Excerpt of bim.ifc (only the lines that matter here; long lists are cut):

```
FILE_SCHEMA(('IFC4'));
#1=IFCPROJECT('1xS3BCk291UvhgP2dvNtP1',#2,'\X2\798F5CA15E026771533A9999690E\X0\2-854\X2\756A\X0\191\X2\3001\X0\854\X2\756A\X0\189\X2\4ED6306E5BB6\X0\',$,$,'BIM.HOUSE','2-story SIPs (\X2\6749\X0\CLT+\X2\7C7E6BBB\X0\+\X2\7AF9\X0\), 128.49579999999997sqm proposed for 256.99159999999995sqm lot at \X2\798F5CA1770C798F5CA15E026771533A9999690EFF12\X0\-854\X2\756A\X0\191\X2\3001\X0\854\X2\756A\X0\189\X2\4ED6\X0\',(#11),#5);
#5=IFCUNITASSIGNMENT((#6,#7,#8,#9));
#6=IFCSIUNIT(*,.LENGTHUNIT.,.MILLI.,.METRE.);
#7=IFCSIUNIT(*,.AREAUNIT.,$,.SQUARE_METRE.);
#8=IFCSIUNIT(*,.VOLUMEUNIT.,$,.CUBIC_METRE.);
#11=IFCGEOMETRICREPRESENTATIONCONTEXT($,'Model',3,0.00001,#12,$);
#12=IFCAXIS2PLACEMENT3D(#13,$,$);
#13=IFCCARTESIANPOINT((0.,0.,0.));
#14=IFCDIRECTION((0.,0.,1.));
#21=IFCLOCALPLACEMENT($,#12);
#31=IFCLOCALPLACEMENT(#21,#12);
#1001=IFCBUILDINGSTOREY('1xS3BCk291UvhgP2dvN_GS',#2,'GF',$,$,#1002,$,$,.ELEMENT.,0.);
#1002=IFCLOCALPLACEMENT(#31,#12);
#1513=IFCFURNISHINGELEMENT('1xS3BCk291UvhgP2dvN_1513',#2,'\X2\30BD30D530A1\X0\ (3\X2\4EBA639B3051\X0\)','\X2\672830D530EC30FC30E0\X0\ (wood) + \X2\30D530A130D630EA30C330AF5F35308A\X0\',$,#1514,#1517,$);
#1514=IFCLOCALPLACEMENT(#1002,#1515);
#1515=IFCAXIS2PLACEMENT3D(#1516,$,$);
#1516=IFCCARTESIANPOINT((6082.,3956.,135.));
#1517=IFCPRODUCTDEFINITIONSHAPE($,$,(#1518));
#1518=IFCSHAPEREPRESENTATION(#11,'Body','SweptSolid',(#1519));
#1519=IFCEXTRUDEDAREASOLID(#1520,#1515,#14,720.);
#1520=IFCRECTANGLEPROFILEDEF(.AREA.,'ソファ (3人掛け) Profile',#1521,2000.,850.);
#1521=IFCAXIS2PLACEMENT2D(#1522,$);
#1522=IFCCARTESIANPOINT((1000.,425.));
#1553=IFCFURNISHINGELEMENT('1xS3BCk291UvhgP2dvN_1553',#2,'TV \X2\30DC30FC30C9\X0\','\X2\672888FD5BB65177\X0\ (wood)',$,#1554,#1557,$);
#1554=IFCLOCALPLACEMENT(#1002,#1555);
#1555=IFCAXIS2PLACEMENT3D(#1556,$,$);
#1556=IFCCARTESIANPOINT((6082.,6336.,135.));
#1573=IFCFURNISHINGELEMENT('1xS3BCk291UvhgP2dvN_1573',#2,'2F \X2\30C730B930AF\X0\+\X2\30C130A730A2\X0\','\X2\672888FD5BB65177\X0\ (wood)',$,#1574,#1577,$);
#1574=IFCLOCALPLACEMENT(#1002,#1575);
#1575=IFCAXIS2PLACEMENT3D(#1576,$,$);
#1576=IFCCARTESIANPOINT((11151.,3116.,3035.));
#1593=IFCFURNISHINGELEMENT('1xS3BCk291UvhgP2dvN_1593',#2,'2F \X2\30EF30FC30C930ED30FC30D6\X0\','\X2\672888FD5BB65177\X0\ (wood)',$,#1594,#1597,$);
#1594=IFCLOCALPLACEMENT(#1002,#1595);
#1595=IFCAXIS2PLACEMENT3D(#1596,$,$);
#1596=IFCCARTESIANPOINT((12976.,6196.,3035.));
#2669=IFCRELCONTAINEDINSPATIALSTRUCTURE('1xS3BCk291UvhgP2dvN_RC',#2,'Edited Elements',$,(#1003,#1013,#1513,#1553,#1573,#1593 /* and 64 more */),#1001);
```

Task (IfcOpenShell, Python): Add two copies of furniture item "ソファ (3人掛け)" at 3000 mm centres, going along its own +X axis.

```python
import ifcopenshell
import ifcopenshell.api.geometry
import ifcopenshell.api.root
import ifcopenshell.util.element
import ifcopenshell.util.placement
import ifcopenshell.util.unit

model = ifcopenshell.open("bim.ifc")
unit_scale = ifcopenshell.util.unit.calculate_unit_scale(model)


def reuse_history(source, copy):
    """copy_class also copies each property set's owner history, people and application; keep the originals."""
    for rel in copy.IsDefinedBy:
        if rel.is_a("IfcRelDefinesByProperties") and (history := rel.RelatingPropertyDefinition.OwnerHistory):
            rel.RelatingPropertyDefinition.OwnerHistory = source.OwnerHistory
            ifcopenshell.util.element.remove_deep2(model, history)


source = model.by_guid("1xS3BCk291UvhgP2dvN_1513")
base = ifcopenshell.util.placement.get_local_placement(source.ObjectPlacement)
step = base[:3, 0] * 3 / unit_scale

for i in range(1, 3):
    copy = ifcopenshell.api.root.copy_class(model, product=source)
    copy.Representation = ifcopenshell.util.element.copy_deep(
        model, source.Representation, exclude=["IfcGeometricRepresentationContext", "IfcRepresentationMap"]
    )
    reuse_history(source, copy)
    matrix = base.copy()
    matrix[:3, 3] += i * step
    print("added at", matrix[:3, 3].round(3) + 0.0)
    ifcopenshell.api.geometry.edit_object_placement(model, product=copy, matrix=matrix, is_si=False)

model.write("bim_rev.ifc")
```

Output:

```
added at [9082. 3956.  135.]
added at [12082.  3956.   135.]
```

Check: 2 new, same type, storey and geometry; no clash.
